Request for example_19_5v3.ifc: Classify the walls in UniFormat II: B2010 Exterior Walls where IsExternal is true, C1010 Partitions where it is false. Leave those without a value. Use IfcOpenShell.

First a look at what the model holds.

```python
import ifcopenshell
import ifcopenshell.util.element

model = ifcopenshell.open("example_19_5v3.ifc")
print(model.schema)
print("classifications:", [c.Name for c in model.by_type("IfcClassification")])
values = [ifcopenshell.util.element.get_pset(e, "Pset_WallCommon", "IsExternal") for e in model.by_type("IfcWall")]
for value in (True, False, None):
    print("IsExternal", value, values.count(value))
```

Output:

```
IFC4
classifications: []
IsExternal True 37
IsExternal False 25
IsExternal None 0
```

```python
import ifcopenshell
import ifcopenshell.api.classification
import ifcopenshell.util.element

model = ifcopenshell.open("example_19_5v3.ifc")

system = ifcopenshell.api.classification.add_classification(model, classification="UniFormat II")

walls = model.by_type("IfcWall")
external = {e: ifcopenshell.util.element.get_pset(e, "Pset_WallCommon", "IsExternal") for e in walls}
for flag, code, name in ((True, "B2010", "Exterior Walls"), (False, "C1010", "Partitions")):
    products = [e for e in walls if external[e] is flag]
    ifcopenshell.api.classification.add_reference(
        model, products=products, classification=system, identification=code, name=name
    )
    print(code, len(products))

model.write("example_19_5v3_edited.ifc")
```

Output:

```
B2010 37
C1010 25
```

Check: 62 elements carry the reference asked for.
